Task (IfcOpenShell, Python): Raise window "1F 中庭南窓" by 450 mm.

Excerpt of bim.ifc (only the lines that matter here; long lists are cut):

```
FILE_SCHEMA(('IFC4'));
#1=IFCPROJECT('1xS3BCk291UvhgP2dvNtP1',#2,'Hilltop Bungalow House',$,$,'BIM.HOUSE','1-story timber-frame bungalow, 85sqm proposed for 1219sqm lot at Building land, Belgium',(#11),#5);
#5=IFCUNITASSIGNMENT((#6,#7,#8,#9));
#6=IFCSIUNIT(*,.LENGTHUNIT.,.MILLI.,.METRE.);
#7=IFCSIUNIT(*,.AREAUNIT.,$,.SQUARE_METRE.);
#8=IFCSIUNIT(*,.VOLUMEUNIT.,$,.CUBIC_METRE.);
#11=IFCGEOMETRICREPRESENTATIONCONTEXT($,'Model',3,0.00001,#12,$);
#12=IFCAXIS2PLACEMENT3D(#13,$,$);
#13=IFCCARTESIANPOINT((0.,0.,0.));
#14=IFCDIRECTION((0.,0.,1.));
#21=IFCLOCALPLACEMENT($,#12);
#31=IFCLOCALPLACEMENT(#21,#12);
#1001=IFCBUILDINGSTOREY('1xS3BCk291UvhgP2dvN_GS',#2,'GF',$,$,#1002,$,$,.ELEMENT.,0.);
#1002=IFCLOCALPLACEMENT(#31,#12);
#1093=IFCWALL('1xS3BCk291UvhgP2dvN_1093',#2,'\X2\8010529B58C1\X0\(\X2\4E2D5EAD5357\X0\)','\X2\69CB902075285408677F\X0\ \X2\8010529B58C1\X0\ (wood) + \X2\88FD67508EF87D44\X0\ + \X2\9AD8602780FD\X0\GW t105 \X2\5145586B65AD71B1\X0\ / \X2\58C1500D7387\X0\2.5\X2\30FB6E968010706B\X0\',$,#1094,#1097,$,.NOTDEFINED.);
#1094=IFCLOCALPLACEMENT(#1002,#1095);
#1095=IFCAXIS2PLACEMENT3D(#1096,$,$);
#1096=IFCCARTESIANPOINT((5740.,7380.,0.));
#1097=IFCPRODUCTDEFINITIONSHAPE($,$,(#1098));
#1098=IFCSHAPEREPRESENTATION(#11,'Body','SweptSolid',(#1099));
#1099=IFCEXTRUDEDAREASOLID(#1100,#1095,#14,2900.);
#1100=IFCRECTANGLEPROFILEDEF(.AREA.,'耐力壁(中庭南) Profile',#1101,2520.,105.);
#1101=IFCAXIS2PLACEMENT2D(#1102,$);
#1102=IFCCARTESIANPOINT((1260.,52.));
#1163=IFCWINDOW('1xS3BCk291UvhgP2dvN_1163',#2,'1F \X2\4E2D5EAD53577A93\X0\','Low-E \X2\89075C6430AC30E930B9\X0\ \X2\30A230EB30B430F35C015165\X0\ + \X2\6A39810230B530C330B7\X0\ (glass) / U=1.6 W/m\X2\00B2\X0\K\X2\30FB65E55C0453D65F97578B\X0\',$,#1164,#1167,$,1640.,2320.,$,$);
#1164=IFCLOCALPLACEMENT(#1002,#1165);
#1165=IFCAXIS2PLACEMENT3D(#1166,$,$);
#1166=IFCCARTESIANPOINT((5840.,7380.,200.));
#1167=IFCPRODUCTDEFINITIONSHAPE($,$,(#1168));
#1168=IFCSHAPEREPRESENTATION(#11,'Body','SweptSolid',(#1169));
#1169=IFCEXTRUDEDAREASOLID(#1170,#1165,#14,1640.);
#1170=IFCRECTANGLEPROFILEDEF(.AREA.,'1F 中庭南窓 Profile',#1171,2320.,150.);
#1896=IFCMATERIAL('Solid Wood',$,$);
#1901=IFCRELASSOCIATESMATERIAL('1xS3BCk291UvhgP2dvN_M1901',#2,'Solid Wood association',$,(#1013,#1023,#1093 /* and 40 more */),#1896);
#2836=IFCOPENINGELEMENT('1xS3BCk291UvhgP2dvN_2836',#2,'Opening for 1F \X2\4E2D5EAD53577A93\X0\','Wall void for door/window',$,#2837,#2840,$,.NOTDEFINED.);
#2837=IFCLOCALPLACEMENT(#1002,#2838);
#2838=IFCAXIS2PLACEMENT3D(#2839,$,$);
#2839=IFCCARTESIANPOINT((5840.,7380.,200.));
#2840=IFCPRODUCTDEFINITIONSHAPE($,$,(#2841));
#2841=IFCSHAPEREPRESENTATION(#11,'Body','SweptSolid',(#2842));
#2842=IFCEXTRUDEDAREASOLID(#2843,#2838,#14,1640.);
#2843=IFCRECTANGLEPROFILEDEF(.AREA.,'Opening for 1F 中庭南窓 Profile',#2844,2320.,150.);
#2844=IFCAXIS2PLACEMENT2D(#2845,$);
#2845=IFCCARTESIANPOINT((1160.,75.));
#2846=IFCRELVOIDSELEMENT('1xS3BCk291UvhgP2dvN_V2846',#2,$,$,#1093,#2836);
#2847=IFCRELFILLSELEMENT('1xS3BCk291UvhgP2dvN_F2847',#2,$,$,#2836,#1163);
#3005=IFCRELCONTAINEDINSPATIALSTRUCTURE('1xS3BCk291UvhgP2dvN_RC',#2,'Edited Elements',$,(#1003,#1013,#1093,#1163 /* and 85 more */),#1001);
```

```python
import numpy as np
import ifcopenshell
import ifcopenshell.api.geometry
import ifcopenshell.util.placement
import ifcopenshell.util.unit

model = ifcopenshell.open("bim.ifc")
unit_scale = ifcopenshell.util.unit.calculate_unit_scale(model)

window = model.by_id(1163)
opening = window.FillsVoids[0].RelatingOpeningElement
dz = 0.45 / unit_scale

shift = np.array([0.0, 0.0, dz])
# The window is not placed relative to its opening, so move both.
for product in (opening, window):
    matrix = ifcopenshell.util.placement.get_local_placement(product.ObjectPlacement)
    matrix[:3, 3] += shift
    ifcopenshell.api.geometry.edit_object_placement(model, product=product, matrix=matrix, is_si=False)

print(f"moved by {dz * unit_scale:+.3f} m")

model.write("bim-out.ifc")
```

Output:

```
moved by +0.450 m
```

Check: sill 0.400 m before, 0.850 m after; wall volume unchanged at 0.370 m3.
